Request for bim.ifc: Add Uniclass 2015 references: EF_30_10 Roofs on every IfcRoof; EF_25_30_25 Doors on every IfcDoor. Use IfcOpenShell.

First a look at what the model holds.

```python
import ifcopenshell

model = ifcopenshell.open("bim.ifc")
print(model.schema)
print("classifications:", [c.Name for c in model.by_type("IfcClassification")])
for ifc_class in ("IfcDoor", "IfcRoof", "IfcStair", "IfcWall", "IfcWindow"):
    print(ifc_class, len(model.by_type(ifc_class)))
```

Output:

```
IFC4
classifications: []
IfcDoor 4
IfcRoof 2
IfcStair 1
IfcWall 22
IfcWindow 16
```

```python
import ifcopenshell
import ifcopenshell.api.classification

model = ifcopenshell.open("bim.ifc")

system = ifcopenshell.api.classification.add_classification(model, classification="Uniclass 2015")

codes = {
    "IfcRoof": ("EF_30_10", "Roofs"),
    "IfcDoor": ("EF_25_30_25", "Doors"),
}
for ifc_class, (code, name) in codes.items():
    products = model.by_type(ifc_class)
    ifcopenshell.api.classification.add_reference(
        model, products=products, classification=system, identification=code, name=name
    )
    print(code, len(products))

model.write("bim_rev.ifc")
```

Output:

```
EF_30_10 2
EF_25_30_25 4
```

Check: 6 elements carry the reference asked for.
